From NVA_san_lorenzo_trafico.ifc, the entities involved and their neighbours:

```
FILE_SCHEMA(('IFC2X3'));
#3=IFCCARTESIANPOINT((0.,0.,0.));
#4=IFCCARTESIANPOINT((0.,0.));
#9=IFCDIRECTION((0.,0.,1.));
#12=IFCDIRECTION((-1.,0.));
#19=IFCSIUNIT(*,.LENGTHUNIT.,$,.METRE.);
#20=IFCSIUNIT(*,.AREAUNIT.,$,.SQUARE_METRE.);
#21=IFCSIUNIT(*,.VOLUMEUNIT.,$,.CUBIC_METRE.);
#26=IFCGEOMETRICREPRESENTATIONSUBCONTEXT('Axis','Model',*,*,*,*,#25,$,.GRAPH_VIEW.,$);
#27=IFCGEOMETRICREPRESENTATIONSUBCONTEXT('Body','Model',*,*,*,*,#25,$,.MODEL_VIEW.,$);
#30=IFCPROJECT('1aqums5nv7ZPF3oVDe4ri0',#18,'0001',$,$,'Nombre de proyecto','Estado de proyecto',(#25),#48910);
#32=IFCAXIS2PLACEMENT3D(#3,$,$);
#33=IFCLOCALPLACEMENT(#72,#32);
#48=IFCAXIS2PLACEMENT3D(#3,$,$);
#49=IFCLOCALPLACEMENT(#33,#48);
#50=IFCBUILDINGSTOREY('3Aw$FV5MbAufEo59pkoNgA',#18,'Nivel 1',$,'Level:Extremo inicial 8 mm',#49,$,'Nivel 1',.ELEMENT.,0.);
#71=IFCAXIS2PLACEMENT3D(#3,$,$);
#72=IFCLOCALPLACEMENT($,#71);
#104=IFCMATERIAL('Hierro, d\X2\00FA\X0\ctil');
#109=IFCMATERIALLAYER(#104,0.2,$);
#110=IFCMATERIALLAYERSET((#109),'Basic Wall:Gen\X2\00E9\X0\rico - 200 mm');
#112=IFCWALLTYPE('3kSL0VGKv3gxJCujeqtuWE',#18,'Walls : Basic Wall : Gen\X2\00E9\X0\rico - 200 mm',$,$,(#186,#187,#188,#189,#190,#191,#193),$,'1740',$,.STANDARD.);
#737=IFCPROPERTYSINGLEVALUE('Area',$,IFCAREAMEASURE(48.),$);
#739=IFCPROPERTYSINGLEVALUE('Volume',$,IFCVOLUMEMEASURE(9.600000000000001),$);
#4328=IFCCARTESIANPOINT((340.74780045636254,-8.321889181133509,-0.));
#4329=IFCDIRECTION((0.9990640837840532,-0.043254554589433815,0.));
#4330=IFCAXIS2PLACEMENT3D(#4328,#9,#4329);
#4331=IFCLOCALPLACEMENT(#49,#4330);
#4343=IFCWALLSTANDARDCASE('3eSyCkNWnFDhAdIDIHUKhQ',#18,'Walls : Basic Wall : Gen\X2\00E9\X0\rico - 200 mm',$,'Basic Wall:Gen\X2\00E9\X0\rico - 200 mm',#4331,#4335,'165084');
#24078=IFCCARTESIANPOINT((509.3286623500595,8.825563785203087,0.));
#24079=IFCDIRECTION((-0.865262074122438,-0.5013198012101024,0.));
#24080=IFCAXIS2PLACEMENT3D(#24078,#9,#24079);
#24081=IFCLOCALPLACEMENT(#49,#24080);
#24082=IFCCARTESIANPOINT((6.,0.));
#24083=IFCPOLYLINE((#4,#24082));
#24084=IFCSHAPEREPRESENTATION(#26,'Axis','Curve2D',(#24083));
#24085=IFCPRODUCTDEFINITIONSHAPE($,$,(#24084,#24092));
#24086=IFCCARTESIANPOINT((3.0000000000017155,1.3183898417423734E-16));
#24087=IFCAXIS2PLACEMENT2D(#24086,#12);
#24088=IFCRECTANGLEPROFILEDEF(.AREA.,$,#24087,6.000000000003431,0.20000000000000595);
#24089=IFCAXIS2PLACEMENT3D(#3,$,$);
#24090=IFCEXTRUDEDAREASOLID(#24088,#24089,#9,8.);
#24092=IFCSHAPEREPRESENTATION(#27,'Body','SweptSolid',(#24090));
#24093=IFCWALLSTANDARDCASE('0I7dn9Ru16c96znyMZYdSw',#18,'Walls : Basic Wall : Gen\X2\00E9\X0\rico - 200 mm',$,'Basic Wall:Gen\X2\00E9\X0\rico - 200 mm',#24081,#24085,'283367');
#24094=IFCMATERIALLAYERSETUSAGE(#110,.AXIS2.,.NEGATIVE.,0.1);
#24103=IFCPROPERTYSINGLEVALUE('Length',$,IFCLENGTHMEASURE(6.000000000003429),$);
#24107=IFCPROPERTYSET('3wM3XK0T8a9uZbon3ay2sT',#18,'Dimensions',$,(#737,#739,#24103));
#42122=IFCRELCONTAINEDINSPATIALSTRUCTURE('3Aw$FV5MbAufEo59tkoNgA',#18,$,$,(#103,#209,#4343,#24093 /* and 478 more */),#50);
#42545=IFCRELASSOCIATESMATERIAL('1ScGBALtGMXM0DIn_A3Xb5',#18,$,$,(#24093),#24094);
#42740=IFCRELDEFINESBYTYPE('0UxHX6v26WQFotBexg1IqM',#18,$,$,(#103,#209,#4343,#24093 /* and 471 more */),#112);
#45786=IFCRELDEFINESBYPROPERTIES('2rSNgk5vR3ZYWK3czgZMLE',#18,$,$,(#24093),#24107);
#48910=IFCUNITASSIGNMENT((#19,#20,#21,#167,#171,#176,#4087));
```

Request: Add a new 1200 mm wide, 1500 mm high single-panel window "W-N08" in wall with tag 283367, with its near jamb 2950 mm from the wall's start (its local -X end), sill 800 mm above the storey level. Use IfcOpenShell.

```python
import numpy as np
import ifcopenshell
import ifcopenshell.api.feature
import ifcopenshell.api.geometry
import ifcopenshell.api.pset
import ifcopenshell.api.root
import ifcopenshell.api.spatial
import ifcopenshell.api.type
import ifcopenshell.geom
import ifcopenshell.util.element
import ifcopenshell.util.placement
import ifcopenshell.util.representation
import ifcopenshell.util.shape
import ifcopenshell.util.unit

model = ifcopenshell.open("NVA_san_lorenzo_trafico.ifc")
unit_scale = ifcopenshell.util.unit.calculate_unit_scale(model)
area_scale = ifcopenshell.util.unit.calculate_unit_scale(model, "AREAUNIT")
volume_scale = ifcopenshell.util.unit.calculate_unit_scale(model, "VOLUMEUNIT")
settings = ifcopenshell.geom.settings()


def volume(element):
    """Net volume in cubic metres, openings subtracted."""
    shape = ifcopenshell.geom.create_shape(settings, element)
    return ifcopenshell.util.shape.get_volume(shape.geometry)


wall = model.by_id(24093)
storey = ifcopenshell.util.element.get_container(wall, ifc_class="IfcBuildingStorey")
context = ifcopenshell.util.representation.get_context(model, "Model", "Body", "MODEL_VIEW")
before = volume(wall)

width, height, from_end, sill = 1.2, 1.5, 2.95, 0.8  # metres

# The wall runs along its own X axis, and the end named is its -X end.
wall_shape = ifcopenshell.geom.create_shape(settings, wall)
x, y, z = ifcopenshell.util.shape.get_vertices(wall_shape.geometry).T
start = x.min() + from_end
face, thickness = float(y.min()), float(y.max() - y.min())
wall_matrix = ifcopenshell.util.placement.get_local_placement(wall.ObjectPlacement)
level = ifcopenshell.util.placement.get_local_placement(storey.ObjectPlacement)[2, 3]


def in_wall(x, y):
    """Placement at x, y metres in the wall's axes, at sill height."""
    matrix = wall_matrix.copy()
    matrix[:, 3] = wall_matrix @ np.array([x / unit_scale, y / unit_scale, 0.0, 1.0])
    matrix[2, 3] = level + sill / unit_scale
    return matrix


# Opening: a box that overshoots both wall faces by 50 mm.
opening = ifcopenshell.api.root.create_entity(model, ifc_class="IfcOpeningElement")
box = ifcopenshell.api.geometry.add_wall_representation(
    model, context=context, length=width, height=height, thickness=thickness + 0.1
)
ifcopenshell.api.geometry.assign_representation(model, product=opening, representation=box)
ifcopenshell.api.geometry.edit_object_placement(model, product=opening, matrix=in_wall(start, face - 0.05), is_si=False)
ifcopenshell.api.feature.add_feature(model, feature=opening, element=wall)

window = ifcopenshell.api.root.create_entity(model, ifc_class="IfcWindow", name="W-N08")
window.OverallWidth, window.OverallHeight = width / unit_scale, height / unit_scale
body = ifcopenshell.api.geometry.add_window_representation(
    model,
    context=context,
    overall_width=window.OverallWidth,
    overall_height=window.OverallHeight,
    partition_type="SINGLE_PANEL",
)
ifcopenshell.api.geometry.assign_representation(model, product=window, representation=body)
ifcopenshell.api.spatial.assign_container(model, products=[window], relating_structure=storey)
fills = ifcopenshell.api.feature.add_filling(model, opening=opening, element=window)
fills.OwnerHistory = window.OwnerHistory  # required in IFC2X3

# IFC2X3 keeps the operation on the window style.
style = ifcopenshell.api.root.create_entity(model, ifc_class="IfcWindowStyle", name="W-N08")
style.OperationType, style.ConstructionType = "SINGLE_PANEL", "NOTDEFINED"
style.ParameterTakesPrecedence = style.Sizeable = False
ifcopenshell.api.type.assign_type(model, related_objects=[window], relating_type=style)

# Centre the window in the wall's thickness.
ifcopenshell.api.geometry.edit_object_placement(model, product=window, matrix=in_wall(start, face), is_si=False)
window_shape = ifcopenshell.geom.create_shape(settings, window)
depth = ifcopenshell.util.shape.get_vertices(window_shape.geometry)[:, 1]
offset = face + thickness / 2 - (depth.min() + depth.max()) / 2
ifcopenshell.api.geometry.edit_object_placement(model, product=window, matrix=in_wall(start, offset), is_si=False)

after = volume(wall)

# Update the wall's stored quantities.
pset = model.by_id(ifcopenshell.util.element.get_pset(wall, "Dimensions", should_inherit=False)["id"])
ifcopenshell.api.pset.edit_pset(model, pset=pset, properties={
    "Area": model.create_entity("IfcAreaMeasure", after / thickness / area_scale),
    "Volume": model.create_entity("IfcVolumeMeasure", after / volume_scale),
})

print(f"wall volume {before:.3f} -> {after:.3f} m3")

model.write("NVA_san_lorenzo_trafico_rev.ifc")
```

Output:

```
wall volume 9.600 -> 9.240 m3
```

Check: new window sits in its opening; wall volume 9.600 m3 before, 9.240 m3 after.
